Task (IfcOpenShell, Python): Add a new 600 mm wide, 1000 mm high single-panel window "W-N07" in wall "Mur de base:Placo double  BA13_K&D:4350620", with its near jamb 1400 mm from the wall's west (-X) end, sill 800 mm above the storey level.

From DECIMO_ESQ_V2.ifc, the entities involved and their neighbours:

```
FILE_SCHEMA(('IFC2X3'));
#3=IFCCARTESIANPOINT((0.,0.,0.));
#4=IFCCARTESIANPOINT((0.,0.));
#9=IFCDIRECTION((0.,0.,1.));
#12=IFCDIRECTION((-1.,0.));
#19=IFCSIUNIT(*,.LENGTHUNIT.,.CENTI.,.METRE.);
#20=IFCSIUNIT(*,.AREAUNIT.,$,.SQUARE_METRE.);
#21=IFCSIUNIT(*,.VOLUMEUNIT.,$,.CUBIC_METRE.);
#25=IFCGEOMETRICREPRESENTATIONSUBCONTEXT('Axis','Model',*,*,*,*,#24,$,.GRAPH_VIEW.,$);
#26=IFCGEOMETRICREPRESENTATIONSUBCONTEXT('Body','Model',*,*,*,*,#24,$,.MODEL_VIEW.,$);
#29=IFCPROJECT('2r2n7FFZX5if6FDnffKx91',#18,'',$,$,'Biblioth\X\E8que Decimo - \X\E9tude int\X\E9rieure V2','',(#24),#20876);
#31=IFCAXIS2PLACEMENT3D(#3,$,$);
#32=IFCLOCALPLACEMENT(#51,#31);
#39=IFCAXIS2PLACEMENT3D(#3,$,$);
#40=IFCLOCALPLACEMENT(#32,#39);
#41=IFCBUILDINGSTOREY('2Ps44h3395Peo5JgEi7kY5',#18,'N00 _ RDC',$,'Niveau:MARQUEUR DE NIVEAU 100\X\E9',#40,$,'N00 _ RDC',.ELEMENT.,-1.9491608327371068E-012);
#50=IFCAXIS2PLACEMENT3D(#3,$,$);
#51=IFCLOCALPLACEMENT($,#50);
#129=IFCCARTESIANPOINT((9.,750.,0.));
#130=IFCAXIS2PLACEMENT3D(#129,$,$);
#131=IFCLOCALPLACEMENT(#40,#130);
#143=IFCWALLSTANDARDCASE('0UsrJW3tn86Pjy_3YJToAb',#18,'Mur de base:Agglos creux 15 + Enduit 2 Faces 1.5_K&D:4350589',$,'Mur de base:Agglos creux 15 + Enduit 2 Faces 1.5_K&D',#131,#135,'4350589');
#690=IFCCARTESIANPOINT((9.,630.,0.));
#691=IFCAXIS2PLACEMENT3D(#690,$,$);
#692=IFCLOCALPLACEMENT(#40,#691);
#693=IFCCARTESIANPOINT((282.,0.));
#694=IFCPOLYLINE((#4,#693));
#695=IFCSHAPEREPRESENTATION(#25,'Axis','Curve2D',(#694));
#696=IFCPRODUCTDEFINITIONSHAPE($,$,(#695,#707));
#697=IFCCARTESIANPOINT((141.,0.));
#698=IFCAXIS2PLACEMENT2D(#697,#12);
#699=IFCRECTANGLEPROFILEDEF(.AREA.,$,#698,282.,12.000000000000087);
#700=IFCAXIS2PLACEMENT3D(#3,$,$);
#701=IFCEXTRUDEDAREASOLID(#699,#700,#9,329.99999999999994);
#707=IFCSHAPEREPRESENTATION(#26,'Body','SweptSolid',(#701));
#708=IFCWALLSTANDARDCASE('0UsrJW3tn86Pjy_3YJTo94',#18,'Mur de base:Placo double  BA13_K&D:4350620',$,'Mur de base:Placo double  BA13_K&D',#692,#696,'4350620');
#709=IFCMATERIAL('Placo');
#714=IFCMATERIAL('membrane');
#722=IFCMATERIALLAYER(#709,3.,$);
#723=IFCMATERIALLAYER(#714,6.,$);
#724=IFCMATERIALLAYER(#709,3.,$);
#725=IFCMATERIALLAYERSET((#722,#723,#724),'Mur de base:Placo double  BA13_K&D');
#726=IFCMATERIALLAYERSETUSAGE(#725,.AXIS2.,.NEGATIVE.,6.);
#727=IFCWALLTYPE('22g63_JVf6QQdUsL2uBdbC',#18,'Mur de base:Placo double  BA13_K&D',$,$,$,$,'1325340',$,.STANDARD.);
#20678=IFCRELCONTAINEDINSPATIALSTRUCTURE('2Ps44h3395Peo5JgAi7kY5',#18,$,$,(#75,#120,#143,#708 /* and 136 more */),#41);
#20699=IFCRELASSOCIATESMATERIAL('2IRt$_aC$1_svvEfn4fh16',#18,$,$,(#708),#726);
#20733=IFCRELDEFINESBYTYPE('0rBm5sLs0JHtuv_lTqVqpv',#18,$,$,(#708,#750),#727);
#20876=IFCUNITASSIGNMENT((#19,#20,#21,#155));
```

```python
import numpy as np
import ifcopenshell
import ifcopenshell.api.feature
import ifcopenshell.api.geometry
import ifcopenshell.api.root
import ifcopenshell.api.spatial
import ifcopenshell.api.type
import ifcopenshell.geom
import ifcopenshell.util.element
import ifcopenshell.util.placement
import ifcopenshell.util.representation
import ifcopenshell.util.shape
import ifcopenshell.util.unit

model = ifcopenshell.open("DECIMO_ESQ_V2.ifc")
unit_scale = ifcopenshell.util.unit.calculate_unit_scale(model)
settings = ifcopenshell.geom.settings()


def volume(element):
    """Net volume in cubic metres, openings subtracted."""
    shape = ifcopenshell.geom.create_shape(settings, element)
    return ifcopenshell.util.shape.get_volume(shape.geometry)


wall = model.by_guid("0UsrJW3tn86Pjy_3YJTo94")
storey = ifcopenshell.util.element.get_container(wall, ifc_class="IfcBuildingStorey")
context = ifcopenshell.util.representation.get_context(model, "Model", "Body", "MODEL_VIEW")
before = volume(wall)

width, height, from_end, sill = 0.6, 1, 1.4, 0.8  # metres

# The wall runs along its own X axis, and the end named is its -X end.
wall_shape = ifcopenshell.geom.create_shape(settings, wall)
x, y, z = ifcopenshell.util.shape.get_vertices(wall_shape.geometry).T
start = x.min() + from_end
face, thickness = float(y.min()), float(y.max() - y.min())
wall_matrix = ifcopenshell.util.placement.get_local_placement(wall.ObjectPlacement)
level = ifcopenshell.util.placement.get_local_placement(storey.ObjectPlacement)[2, 3]


def in_wall(x, y):
    """Placement at x, y metres in the wall's axes, at sill height."""
    matrix = wall_matrix.copy()
    matrix[:, 3] = wall_matrix @ np.array([x / unit_scale, y / unit_scale, 0.0, 1.0])
    matrix[2, 3] = level + sill / unit_scale
    return matrix


# Opening: a box that overshoots both wall faces by 50 mm.
opening = ifcopenshell.api.root.create_entity(model, ifc_class="IfcOpeningElement")
box = ifcopenshell.api.geometry.add_wall_representation(
    model, context=context, length=width, height=height, thickness=thickness + 0.1
)
ifcopenshell.api.geometry.assign_representation(model, product=opening, representation=box)
ifcopenshell.api.geometry.edit_object_placement(model, product=opening, matrix=in_wall(start, face - 0.05), is_si=False)
ifcopenshell.api.feature.add_feature(model, feature=opening, element=wall)

window = ifcopenshell.api.root.create_entity(model, ifc_class="IfcWindow", name="W-N07")
window.OverallWidth, window.OverallHeight = width / unit_scale, height / unit_scale
body = ifcopenshell.api.geometry.add_window_representation(
    model,
    context=context,
    overall_width=window.OverallWidth,
    overall_height=window.OverallHeight,
    partition_type="SINGLE_PANEL",
)
ifcopenshell.api.geometry.assign_representation(model, product=window, representation=body)
ifcopenshell.api.spatial.assign_container(model, products=[window], relating_structure=storey)
fills = ifcopenshell.api.feature.add_filling(model, opening=opening, element=window)
fills.OwnerHistory = window.OwnerHistory  # required in IFC2X3

# IFC2X3 keeps the operation on the window style.
style = ifcopenshell.api.root.create_entity(model, ifc_class="IfcWindowStyle", name="W-N07")
style.OperationType, style.ConstructionType = "SINGLE_PANEL", "NOTDEFINED"
style.ParameterTakesPrecedence = style.Sizeable = False
ifcopenshell.api.type.assign_type(model, related_objects=[window], relating_type=style)

# Centre the window in the wall's thickness.
ifcopenshell.api.geometry.edit_object_placement(model, product=window, matrix=in_wall(start, face), is_si=False)
window_shape = ifcopenshell.geom.create_shape(settings, window)
depth = ifcopenshell.util.shape.get_vertices(window_shape.geometry)[:, 1]
offset = face + thickness / 2 - (depth.min() + depth.max()) / 2
ifcopenshell.api.geometry.edit_object_placement(model, product=window, matrix=in_wall(start, offset), is_si=False)

after = volume(wall)

print(f"wall volume {before:.3f} -> {after:.3f} m3")

model.write("DECIMO_ESQ_V2_updated.ifc")
```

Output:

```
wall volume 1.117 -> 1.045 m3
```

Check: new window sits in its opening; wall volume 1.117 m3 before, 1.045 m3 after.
